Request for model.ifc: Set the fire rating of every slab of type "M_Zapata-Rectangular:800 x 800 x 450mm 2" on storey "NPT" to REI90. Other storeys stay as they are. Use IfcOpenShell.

First a look at what the model holds.

```python
import ifcopenshell
import ifcopenshell.util.element

model = ifcopenshell.open("model.ifc")
print(model.schema)
storey = next(s for s in model.by_type("IfcBuildingStorey") if s.Name == "NPT")
slabs = [e for e in ifcopenshell.util.element.get_decomposition(storey) if e.is_a("IfcSlab")]
seen = {}
for e in slabs:
    element_type = ifcopenshell.util.element.get_type(e)
    key = (element_type.Name if element_type != e and element_type else None, ifcopenshell.util.element.get_pset(e, "Pset_SlabCommon", "FireRating"))
    seen[key] = seen.get(key, 0) + 1
for (name, value), count in sorted(seen.items(), key=str):
    print(count, "x", name, "|", value)
```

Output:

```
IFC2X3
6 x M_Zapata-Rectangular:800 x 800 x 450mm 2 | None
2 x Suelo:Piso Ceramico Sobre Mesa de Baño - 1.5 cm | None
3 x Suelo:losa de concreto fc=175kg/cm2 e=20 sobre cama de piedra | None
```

```python
import ifcopenshell
import ifcopenshell.api.pset
import ifcopenshell.util.element

model = ifcopenshell.open("model.ifc")

storey = next(s for s in model.by_type("IfcBuildingStorey") if s.Name == "NPT")
slabs = [e for e in ifcopenshell.util.element.get_decomposition(storey) if e.is_a("IfcSlab")]

count = 0
for e in slabs:
    element_type = ifcopenshell.util.element.get_type(e)
    if element_type in (None, e) or element_type.Name != "M_Zapata-Rectangular:800 x 800 x 450mm 2":
        continue
    # add_pset returns the element's existing set when there is one.
    pset = ifcopenshell.api.pset.add_pset(model, product=e, name="Pset_SlabCommon")
    ifcopenshell.api.pset.edit_pset(model, pset=pset, properties={"FireRating": "REI90"})
    count += 1

print(count, "slabs updated")

model.write("model_updated.ifc")
```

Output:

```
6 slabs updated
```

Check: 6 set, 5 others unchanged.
